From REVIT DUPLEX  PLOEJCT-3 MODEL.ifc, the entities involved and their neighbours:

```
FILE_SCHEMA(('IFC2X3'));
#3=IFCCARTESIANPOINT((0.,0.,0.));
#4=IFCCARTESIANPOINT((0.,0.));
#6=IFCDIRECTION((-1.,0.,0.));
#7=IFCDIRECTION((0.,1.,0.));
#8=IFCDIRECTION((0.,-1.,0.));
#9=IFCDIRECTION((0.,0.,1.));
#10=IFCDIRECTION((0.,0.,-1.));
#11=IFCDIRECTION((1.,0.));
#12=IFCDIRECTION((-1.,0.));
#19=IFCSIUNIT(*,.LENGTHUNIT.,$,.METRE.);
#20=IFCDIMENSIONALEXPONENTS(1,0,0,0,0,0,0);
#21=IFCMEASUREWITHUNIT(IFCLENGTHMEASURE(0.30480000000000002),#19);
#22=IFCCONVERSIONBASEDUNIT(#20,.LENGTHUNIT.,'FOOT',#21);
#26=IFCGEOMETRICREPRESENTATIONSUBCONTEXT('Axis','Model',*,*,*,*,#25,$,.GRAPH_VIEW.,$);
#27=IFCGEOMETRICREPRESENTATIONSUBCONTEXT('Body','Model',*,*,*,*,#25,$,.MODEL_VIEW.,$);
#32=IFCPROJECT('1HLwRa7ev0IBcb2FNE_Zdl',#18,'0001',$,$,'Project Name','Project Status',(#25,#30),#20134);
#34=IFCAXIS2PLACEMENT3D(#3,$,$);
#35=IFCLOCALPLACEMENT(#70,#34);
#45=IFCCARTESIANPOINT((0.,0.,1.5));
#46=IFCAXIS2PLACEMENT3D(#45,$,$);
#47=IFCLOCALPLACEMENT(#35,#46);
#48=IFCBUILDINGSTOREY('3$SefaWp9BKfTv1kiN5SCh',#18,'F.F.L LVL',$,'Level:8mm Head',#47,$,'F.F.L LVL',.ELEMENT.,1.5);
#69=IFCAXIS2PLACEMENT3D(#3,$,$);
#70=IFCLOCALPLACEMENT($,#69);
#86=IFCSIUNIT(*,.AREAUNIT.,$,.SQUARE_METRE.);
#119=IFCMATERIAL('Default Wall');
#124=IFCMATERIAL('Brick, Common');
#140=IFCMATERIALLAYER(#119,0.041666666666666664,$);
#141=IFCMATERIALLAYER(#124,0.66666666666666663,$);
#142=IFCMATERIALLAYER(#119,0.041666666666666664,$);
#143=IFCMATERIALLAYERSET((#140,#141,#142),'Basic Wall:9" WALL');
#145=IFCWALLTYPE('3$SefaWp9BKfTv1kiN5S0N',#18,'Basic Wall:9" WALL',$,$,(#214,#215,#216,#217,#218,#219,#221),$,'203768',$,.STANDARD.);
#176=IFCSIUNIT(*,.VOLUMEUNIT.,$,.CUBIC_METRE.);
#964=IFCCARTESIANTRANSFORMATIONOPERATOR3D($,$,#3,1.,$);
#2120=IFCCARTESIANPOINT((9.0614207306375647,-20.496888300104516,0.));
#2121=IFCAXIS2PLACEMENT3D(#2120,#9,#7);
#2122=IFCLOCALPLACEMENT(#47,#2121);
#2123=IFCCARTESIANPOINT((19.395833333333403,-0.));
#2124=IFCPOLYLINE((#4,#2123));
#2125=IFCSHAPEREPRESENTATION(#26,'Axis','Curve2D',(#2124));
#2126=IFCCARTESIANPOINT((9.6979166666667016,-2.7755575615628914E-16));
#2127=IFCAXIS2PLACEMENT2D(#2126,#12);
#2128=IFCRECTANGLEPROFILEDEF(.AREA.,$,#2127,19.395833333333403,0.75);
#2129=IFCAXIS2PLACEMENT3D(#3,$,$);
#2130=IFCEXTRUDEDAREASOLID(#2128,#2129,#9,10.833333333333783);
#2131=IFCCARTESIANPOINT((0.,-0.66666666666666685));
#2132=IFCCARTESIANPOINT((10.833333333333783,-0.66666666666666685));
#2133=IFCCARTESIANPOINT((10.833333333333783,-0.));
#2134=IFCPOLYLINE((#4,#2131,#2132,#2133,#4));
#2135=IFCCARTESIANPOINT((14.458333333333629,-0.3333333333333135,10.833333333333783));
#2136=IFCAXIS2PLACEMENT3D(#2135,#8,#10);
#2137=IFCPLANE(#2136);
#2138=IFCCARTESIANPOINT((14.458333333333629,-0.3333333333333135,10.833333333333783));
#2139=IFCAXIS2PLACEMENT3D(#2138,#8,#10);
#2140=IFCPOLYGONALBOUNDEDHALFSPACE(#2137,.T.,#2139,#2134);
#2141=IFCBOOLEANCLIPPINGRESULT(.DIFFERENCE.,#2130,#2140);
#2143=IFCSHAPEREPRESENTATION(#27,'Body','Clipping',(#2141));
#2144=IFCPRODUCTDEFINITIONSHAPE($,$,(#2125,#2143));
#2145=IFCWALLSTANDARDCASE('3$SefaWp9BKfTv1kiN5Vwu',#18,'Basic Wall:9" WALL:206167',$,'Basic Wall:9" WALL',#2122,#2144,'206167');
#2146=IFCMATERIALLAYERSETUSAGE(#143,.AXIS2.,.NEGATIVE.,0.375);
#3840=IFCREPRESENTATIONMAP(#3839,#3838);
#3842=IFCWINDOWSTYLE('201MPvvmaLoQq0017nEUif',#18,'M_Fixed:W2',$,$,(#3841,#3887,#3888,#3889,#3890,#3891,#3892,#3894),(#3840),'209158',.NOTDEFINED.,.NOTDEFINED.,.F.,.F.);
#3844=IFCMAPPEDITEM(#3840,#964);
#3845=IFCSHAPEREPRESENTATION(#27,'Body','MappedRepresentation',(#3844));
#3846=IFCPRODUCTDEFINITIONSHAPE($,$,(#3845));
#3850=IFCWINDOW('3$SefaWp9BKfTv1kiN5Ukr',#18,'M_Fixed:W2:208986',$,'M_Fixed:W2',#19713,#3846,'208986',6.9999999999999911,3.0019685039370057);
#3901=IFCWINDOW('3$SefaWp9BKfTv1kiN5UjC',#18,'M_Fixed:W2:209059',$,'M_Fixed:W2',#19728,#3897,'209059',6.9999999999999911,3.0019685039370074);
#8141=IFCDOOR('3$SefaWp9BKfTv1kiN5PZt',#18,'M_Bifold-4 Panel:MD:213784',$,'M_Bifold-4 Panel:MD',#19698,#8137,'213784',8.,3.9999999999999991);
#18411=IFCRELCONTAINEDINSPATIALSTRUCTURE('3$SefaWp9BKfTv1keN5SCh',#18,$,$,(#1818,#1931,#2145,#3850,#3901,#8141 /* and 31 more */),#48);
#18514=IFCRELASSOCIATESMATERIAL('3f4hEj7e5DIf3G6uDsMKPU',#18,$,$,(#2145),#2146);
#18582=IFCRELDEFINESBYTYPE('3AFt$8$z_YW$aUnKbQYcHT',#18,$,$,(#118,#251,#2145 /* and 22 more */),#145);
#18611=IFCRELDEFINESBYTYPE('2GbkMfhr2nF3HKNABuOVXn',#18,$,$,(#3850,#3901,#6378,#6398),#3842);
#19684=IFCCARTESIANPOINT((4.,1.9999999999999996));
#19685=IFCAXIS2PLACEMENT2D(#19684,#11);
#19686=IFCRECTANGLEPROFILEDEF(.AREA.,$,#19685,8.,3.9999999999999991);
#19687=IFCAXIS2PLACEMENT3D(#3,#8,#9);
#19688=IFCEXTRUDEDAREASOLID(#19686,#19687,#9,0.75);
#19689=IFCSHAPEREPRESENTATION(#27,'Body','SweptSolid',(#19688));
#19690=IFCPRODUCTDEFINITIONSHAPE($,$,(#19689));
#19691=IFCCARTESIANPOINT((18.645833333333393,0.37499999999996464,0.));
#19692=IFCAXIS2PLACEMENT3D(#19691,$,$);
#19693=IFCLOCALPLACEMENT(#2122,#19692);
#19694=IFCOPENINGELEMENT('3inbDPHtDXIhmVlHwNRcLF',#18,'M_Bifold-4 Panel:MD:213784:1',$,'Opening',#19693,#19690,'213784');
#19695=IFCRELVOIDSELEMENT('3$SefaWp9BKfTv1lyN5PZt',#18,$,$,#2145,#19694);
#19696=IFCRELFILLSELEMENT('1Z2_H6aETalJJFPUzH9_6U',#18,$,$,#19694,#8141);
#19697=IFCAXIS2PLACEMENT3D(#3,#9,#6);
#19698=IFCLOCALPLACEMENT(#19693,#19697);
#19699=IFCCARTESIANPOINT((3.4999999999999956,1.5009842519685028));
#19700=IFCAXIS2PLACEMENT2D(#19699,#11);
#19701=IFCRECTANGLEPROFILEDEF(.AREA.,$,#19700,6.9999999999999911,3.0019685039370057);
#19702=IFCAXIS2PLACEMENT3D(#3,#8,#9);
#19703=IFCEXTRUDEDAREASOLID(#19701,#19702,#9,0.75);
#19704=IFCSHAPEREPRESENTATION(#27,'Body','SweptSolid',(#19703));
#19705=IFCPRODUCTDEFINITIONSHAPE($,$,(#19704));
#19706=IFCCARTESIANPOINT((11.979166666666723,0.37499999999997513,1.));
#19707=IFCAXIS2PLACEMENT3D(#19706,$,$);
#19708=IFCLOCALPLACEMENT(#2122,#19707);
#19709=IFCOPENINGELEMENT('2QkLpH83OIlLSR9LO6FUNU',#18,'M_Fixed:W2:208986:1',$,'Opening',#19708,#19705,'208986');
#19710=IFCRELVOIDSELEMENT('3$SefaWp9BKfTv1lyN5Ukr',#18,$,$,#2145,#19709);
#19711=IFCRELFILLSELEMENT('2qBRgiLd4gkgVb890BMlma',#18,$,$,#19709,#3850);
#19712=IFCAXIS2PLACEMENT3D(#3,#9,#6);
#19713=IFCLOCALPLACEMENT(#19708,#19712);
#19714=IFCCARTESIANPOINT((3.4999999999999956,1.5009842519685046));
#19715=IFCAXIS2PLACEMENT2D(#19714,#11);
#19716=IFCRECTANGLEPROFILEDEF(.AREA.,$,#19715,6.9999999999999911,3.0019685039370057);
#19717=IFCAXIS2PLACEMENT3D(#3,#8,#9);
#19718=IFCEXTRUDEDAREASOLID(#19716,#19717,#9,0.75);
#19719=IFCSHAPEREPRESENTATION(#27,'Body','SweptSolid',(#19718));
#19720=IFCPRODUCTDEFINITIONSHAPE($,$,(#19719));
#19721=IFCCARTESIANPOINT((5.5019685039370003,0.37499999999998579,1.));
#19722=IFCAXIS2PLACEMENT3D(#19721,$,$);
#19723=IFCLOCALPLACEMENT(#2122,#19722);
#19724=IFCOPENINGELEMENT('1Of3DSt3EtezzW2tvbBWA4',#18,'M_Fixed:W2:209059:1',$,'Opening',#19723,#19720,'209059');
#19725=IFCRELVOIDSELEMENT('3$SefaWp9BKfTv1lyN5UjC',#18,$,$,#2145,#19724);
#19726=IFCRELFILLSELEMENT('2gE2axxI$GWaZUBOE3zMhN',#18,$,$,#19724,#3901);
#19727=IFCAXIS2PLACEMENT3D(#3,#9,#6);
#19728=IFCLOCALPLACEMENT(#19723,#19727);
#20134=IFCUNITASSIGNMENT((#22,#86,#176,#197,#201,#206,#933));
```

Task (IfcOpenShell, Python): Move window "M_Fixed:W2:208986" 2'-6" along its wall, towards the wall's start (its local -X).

```python
import ifcopenshell
import ifcopenshell.api.geometry
import ifcopenshell.util.placement
import ifcopenshell.util.unit

model = ifcopenshell.open("REVIT DUPLEX  PLOEJCT-3 MODEL.ifc")
unit_scale = ifcopenshell.util.unit.calculate_unit_scale(model)

window = model.by_guid("3$SefaWp9BKfTv1kiN5Ukr")
opening = window.FillsVoids[0].RelatingOpeningElement
wall = opening.VoidsElements[0].RelatingBuildingElement

wall_matrix = ifcopenshell.util.placement.get_local_placement(wall.ObjectPlacement)
shift = wall_matrix[:3, 0] * -30 * 0.0254 / unit_scale
before = ifcopenshell.util.placement.get_local_placement(window.ObjectPlacement)[:3, 3].copy()

# The window is placed relative to its opening, so it follows when the opening moves.
matrix = ifcopenshell.util.placement.get_local_placement(opening.ObjectPlacement)
matrix[:3, 3] += shift
ifcopenshell.api.geometry.edit_object_placement(
    model, product=opening, matrix=matrix, is_si=False, should_transform_children=True
)

after = ifcopenshell.util.placement.get_local_placement(window.ObjectPlacement)[:3, 3]
print("window moved by", (after - before).round(3) + 0.0)

model.write("REVIT DUPLEX  PLOEJCT-3 MODEL-out.ifc")
```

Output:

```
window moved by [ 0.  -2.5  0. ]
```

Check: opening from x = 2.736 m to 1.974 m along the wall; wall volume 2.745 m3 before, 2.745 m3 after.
